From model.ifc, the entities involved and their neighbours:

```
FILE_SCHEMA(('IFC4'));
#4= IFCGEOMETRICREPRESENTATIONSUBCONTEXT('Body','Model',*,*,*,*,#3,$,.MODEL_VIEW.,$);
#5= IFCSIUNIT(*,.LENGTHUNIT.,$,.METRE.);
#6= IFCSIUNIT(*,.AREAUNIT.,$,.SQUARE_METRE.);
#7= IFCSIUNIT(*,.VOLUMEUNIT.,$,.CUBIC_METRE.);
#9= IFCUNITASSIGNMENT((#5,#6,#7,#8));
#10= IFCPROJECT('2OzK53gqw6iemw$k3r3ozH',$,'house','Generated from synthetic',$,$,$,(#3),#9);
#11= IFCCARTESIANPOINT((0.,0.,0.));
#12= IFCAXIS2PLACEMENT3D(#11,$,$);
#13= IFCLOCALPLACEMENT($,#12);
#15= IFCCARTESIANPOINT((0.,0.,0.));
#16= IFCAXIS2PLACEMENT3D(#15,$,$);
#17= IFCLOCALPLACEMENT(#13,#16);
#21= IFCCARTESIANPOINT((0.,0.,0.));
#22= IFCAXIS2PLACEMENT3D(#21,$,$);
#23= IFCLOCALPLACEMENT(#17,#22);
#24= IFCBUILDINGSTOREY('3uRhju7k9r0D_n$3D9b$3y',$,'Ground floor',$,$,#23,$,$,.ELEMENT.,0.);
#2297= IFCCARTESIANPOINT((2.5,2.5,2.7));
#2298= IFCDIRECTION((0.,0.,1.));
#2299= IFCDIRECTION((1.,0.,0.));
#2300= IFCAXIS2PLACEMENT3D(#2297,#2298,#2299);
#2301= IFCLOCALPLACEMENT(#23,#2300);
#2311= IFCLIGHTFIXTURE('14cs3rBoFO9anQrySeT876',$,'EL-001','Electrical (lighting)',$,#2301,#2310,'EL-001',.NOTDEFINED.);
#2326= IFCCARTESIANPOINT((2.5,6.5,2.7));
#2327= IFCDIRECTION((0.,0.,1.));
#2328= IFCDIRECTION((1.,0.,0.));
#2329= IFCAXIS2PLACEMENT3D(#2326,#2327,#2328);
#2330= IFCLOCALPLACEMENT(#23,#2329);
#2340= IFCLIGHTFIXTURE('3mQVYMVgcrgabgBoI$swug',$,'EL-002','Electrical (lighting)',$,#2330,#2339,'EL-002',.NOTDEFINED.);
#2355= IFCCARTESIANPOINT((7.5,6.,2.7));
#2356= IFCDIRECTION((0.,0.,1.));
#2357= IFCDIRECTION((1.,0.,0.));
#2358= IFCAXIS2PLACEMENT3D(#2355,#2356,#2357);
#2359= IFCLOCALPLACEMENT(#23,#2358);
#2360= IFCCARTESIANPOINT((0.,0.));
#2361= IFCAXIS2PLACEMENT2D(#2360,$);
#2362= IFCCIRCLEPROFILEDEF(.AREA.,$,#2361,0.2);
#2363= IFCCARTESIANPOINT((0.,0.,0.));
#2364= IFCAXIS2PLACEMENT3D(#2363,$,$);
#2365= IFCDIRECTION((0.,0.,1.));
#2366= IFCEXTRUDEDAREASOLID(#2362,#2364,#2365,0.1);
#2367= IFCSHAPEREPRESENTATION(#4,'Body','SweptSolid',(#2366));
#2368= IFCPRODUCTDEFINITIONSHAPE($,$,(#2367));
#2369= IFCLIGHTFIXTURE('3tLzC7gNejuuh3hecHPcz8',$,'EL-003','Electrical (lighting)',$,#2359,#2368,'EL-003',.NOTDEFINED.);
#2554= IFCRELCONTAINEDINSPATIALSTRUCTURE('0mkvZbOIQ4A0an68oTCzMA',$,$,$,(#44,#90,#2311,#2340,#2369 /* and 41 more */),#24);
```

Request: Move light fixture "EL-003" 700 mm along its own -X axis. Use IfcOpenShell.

```python
import ifcopenshell
import ifcopenshell.api.geometry
import ifcopenshell.util.placement
import ifcopenshell.util.unit

model = ifcopenshell.open("model.ifc")
unit_scale = ifcopenshell.util.unit.calculate_unit_scale(model)

item = model.by_guid("3tLzC7gNejuuh3hecHPcz8")
matrix = ifcopenshell.util.placement.get_local_placement(item.ObjectPlacement)
matrix[:3, 3] -= matrix[:3, 0] * 0.7 / unit_scale
ifcopenshell.api.geometry.edit_object_placement(model, product=item, matrix=matrix, is_si=False)

print(ifcopenshell.util.placement.get_local_placement(item.ObjectPlacement).round(3) + 0.0)

model.write("model-out.ifc")
```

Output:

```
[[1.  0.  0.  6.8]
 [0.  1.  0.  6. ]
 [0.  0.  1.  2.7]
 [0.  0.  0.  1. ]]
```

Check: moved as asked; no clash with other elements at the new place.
